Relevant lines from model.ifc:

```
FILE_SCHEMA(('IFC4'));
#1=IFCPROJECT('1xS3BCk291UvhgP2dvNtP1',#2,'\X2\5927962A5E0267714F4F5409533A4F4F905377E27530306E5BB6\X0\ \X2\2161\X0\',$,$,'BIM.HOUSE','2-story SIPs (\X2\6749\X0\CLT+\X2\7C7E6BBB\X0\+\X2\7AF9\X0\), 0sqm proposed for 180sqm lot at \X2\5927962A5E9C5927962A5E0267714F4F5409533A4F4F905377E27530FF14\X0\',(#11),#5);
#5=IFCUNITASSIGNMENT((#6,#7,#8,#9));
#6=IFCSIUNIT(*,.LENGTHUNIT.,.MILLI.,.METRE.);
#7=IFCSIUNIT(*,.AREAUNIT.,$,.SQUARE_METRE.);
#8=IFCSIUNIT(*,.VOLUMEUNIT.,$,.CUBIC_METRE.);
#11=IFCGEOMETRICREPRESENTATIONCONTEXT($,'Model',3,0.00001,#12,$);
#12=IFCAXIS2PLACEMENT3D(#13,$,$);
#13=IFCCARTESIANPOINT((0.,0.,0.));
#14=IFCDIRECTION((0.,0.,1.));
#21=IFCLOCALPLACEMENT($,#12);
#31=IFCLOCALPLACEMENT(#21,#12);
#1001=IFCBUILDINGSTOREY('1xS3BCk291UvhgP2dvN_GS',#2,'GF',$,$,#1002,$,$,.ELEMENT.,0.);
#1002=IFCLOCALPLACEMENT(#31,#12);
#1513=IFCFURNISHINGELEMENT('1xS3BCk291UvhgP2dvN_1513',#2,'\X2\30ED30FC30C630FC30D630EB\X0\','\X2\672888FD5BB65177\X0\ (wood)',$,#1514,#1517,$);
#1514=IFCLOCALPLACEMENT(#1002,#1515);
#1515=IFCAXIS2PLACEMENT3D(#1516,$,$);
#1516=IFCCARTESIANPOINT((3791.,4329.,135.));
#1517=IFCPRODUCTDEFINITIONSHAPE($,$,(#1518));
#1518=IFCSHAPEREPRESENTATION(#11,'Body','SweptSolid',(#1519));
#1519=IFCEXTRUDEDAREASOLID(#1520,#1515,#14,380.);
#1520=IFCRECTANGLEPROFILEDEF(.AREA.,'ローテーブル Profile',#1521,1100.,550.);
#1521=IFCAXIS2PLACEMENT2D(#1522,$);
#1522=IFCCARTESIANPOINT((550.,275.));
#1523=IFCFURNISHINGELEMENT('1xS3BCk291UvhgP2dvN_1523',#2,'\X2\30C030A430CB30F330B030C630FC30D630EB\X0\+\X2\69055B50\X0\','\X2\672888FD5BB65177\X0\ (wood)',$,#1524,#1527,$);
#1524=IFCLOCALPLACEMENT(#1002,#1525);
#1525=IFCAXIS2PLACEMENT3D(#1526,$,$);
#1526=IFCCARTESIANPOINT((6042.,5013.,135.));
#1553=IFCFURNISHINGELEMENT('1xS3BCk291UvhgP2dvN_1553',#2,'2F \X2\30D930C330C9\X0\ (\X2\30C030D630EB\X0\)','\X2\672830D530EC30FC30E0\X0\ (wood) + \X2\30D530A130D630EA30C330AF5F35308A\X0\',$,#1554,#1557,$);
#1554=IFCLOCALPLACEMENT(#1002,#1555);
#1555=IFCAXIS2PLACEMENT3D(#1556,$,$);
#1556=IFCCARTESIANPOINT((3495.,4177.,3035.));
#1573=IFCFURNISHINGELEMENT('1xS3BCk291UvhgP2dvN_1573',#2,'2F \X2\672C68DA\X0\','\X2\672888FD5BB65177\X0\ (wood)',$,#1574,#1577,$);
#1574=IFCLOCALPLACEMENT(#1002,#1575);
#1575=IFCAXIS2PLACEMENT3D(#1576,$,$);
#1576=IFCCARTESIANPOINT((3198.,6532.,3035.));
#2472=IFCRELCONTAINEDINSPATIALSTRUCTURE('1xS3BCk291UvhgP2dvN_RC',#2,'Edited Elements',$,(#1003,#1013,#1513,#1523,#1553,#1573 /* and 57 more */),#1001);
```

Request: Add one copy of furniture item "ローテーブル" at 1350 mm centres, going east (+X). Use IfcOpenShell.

```python
import numpy as np
import ifcopenshell
import ifcopenshell.api.geometry
import ifcopenshell.api.root
import ifcopenshell.util.element
import ifcopenshell.util.placement
import ifcopenshell.util.unit

model = ifcopenshell.open("model.ifc")
unit_scale = ifcopenshell.util.unit.calculate_unit_scale(model)


def reuse_history(source, copy):
    """copy_class also copies each property set's owner history, people and application; keep the originals."""
    for rel in copy.IsDefinedBy:
        if rel.is_a("IfcRelDefinesByProperties") and (history := rel.RelatingPropertyDefinition.OwnerHistory):
            rel.RelatingPropertyDefinition.OwnerHistory = source.OwnerHistory
            ifcopenshell.util.element.remove_deep2(model, history)


source = model.by_guid("1xS3BCk291UvhgP2dvN_1513")
base = ifcopenshell.util.placement.get_local_placement(source.ObjectPlacement)
step = np.array([1.0, 0.0, 0.0]) * 1.35 / unit_scale

for i in range(1, 2):
    copy = ifcopenshell.api.root.copy_class(model, product=source)
    copy.Representation = ifcopenshell.util.element.copy_deep(
        model, source.Representation, exclude=["IfcGeometricRepresentationContext", "IfcRepresentationMap"]
    )
    reuse_history(source, copy)
    matrix = base.copy()
    matrix[:3, 3] += i * step
    print("added at", matrix[:3, 3].round(3) + 0.0)
    ifcopenshell.api.geometry.edit_object_placement(model, product=copy, matrix=matrix, is_si=False)

model.write("model_v2.ifc")
```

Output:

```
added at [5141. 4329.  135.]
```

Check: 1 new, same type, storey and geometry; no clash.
